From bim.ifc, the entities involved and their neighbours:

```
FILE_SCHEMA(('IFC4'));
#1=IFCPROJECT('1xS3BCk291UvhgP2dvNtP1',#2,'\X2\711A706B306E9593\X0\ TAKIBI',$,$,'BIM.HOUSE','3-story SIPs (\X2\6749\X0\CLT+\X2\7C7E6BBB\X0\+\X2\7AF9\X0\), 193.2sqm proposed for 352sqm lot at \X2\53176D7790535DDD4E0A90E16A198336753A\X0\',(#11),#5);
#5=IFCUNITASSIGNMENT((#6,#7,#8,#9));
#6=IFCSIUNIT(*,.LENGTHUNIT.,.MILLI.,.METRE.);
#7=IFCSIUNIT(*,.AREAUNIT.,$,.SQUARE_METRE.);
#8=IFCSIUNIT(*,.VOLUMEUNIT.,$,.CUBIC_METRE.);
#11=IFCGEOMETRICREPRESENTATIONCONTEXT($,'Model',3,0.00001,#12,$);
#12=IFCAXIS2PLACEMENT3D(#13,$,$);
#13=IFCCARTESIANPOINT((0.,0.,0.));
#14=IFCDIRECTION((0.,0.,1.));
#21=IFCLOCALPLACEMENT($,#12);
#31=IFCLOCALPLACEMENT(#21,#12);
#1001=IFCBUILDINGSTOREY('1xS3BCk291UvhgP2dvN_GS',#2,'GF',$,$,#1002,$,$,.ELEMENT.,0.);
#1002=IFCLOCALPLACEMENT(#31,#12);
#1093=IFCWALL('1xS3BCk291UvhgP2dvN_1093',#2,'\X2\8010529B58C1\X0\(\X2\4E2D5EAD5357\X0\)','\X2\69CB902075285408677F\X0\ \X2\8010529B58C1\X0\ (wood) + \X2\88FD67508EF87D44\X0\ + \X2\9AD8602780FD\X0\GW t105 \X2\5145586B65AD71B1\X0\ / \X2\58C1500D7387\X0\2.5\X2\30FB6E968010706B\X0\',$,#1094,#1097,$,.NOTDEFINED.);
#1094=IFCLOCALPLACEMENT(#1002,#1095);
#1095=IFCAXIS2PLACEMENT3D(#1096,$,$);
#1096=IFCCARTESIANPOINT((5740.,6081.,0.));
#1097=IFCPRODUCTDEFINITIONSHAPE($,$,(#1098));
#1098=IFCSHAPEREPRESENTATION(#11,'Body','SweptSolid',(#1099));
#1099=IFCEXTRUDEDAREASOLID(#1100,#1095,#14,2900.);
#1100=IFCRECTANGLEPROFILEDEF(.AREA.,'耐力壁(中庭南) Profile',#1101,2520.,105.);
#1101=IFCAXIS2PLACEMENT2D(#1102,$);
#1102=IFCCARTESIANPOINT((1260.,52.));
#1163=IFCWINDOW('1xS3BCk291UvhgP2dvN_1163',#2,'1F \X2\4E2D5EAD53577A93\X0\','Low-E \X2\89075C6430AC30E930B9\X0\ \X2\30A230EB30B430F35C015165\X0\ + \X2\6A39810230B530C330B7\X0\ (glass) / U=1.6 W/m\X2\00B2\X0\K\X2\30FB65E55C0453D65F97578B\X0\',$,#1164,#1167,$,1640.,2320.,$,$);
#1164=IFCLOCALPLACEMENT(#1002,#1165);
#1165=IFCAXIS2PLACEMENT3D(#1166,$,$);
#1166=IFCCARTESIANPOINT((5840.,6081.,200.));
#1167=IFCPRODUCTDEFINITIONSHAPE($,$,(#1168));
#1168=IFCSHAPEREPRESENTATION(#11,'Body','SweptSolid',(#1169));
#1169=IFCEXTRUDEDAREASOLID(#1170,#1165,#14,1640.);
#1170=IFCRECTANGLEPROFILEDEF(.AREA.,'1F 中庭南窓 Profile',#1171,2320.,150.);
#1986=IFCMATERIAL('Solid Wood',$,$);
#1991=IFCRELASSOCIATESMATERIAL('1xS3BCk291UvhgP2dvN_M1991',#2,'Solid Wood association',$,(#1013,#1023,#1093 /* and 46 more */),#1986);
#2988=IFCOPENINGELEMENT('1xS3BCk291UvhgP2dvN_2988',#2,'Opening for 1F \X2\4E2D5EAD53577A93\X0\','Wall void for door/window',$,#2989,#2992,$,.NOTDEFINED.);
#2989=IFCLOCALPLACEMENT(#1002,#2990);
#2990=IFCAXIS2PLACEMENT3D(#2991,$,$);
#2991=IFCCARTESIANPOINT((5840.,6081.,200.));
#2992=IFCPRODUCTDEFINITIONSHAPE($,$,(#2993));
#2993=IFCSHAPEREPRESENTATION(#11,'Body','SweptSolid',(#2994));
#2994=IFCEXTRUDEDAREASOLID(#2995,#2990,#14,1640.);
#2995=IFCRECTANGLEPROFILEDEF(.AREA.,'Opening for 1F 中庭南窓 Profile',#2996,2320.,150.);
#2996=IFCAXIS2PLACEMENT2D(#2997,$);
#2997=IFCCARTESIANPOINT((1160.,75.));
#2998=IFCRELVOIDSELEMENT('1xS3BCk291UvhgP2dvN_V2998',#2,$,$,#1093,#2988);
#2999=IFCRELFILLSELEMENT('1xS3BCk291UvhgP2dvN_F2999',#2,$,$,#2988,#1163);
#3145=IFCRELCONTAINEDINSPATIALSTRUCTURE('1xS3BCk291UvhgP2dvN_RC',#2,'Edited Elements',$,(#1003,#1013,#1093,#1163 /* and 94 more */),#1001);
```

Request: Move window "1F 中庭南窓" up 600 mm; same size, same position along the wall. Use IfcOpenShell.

```python
import numpy as np
import ifcopenshell
import ifcopenshell.api.geometry
import ifcopenshell.util.placement
import ifcopenshell.util.unit

model = ifcopenshell.open("bim.ifc")
unit_scale = ifcopenshell.util.unit.calculate_unit_scale(model)

window = model.by_guid("1xS3BCk291UvhgP2dvN_1163")
opening = window.FillsVoids[0].RelatingOpeningElement
dz = 600.0

shift = np.array([0.0, 0.0, dz])
# The window is not placed relative to its opening, so move both.
for product in (opening, window):
    matrix = ifcopenshell.util.placement.get_local_placement(product.ObjectPlacement)
    matrix[:3, 3] += shift
    ifcopenshell.api.geometry.edit_object_placement(model, product=product, matrix=matrix, is_si=False)

print(f"moved by {dz * unit_scale:+.3f} m")

model.write("bim-out.ifc")
```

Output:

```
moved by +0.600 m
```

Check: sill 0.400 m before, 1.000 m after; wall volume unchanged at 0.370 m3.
